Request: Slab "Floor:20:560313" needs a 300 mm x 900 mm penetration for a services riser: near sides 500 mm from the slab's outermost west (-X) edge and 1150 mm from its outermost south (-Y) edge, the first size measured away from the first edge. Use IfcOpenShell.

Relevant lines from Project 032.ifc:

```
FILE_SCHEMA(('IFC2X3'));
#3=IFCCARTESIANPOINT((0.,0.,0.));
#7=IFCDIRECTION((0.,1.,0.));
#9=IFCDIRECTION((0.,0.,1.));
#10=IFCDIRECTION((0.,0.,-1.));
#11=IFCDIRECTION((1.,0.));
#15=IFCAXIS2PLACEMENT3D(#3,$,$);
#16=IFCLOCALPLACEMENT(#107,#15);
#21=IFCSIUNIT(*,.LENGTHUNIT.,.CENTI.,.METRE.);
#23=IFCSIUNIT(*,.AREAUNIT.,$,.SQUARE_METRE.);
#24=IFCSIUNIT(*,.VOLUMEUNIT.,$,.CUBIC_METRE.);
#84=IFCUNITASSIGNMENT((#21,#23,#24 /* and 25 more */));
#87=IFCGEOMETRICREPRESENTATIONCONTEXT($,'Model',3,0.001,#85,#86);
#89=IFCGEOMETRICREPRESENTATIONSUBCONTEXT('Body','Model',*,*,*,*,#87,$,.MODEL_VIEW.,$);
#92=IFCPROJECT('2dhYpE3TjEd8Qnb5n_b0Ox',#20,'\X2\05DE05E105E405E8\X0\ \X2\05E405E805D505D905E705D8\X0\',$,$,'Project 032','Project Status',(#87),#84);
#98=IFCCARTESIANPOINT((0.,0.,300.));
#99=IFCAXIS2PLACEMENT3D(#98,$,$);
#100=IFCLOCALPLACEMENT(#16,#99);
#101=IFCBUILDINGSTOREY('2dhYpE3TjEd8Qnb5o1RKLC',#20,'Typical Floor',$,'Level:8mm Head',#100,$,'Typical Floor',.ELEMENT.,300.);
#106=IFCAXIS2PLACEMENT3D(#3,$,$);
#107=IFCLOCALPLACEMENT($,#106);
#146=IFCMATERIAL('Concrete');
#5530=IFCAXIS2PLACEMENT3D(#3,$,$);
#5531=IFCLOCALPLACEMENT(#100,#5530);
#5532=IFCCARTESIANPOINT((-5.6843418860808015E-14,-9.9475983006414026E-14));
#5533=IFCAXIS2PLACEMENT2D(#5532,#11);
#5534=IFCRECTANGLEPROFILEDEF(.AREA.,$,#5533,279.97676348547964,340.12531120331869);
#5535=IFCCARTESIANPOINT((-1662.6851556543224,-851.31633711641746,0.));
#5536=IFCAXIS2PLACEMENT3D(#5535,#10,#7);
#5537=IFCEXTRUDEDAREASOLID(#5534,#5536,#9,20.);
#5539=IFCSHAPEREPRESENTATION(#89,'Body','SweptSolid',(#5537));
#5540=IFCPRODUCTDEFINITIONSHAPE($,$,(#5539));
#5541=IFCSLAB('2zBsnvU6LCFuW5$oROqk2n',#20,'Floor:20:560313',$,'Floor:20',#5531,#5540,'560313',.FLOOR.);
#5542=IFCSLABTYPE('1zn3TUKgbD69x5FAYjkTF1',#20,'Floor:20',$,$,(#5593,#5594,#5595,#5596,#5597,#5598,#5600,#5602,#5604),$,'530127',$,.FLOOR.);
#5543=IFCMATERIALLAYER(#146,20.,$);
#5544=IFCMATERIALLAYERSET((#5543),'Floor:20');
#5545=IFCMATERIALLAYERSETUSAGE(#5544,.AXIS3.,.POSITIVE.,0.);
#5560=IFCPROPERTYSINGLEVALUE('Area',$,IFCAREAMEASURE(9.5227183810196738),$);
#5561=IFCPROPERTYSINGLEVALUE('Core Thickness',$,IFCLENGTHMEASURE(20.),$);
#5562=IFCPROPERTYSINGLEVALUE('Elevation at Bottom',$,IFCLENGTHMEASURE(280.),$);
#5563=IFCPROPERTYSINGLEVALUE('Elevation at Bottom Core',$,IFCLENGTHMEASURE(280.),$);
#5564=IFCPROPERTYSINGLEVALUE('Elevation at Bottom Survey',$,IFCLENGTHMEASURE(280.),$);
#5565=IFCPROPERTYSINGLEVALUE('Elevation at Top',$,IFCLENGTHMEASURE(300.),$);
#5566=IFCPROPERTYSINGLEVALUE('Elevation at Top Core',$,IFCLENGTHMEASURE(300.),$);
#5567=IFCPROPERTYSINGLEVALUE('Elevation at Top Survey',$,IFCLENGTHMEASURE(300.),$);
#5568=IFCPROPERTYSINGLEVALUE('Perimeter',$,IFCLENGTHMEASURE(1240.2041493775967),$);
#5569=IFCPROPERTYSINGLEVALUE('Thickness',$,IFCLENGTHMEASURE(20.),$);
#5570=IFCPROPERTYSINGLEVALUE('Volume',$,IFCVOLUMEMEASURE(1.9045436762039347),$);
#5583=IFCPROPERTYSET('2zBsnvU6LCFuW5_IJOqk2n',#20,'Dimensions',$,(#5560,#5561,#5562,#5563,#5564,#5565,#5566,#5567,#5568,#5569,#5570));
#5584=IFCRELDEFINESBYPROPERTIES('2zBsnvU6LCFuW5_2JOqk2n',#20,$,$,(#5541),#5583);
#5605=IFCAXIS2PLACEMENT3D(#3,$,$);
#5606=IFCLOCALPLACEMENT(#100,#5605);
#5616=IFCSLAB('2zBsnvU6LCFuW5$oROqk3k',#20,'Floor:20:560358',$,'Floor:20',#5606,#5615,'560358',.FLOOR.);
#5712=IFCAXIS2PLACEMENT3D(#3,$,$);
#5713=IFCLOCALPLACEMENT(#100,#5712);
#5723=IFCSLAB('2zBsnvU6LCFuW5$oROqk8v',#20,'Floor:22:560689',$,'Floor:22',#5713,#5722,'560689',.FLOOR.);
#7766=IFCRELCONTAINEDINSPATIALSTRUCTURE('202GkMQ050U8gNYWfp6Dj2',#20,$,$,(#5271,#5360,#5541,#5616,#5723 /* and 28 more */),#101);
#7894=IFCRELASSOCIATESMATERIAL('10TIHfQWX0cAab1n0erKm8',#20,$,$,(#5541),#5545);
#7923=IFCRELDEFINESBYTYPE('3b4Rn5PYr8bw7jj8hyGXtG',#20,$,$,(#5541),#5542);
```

```python
import numpy as np
import ifcopenshell
import ifcopenshell.api.feature
import ifcopenshell.api.geometry
import ifcopenshell.api.pset
import ifcopenshell.api.root
import ifcopenshell.geom
import ifcopenshell.util.element
import ifcopenshell.util.placement
import ifcopenshell.util.representation
import ifcopenshell.util.shape
import ifcopenshell.util.unit

model = ifcopenshell.open("Project 032.ifc")
unit_scale = ifcopenshell.util.unit.calculate_unit_scale(model)
area_scale = ifcopenshell.util.unit.calculate_unit_scale(model, "AREAUNIT")
volume_scale = ifcopenshell.util.unit.calculate_unit_scale(model, "VOLUMEUNIT")
settings = ifcopenshell.geom.settings()


def volume(element):
    """Net volume in cubic metres, openings subtracted."""
    shape = ifcopenshell.geom.create_shape(settings, element)
    return ifcopenshell.util.shape.get_volume(shape.geometry)


slab = model.by_guid("2zBsnvU6LCFuW5$oROqk2n")
before = volume(slab)

# Extent in the slab's own axes, in metres. The edges named are its -X and -Y sides.
slab_shape = ifcopenshell.geom.create_shape(settings, slab)
vertices = ifcopenshell.util.shape.get_vertices(slab_shape.geometry)
x_min, y_min, bottom = vertices.min(axis=0)
top = vertices[:, 2].max()

opening = ifcopenshell.api.root.create_entity(model, ifc_class="IfcOpeningElement", name="Services riser opening")
context = ifcopenshell.util.representation.get_context(model, "Model", "Body", "MODEL_VIEW")
width, depth = 0.3, 0.9
outline = [(0.0, 0.0), (width, 0.0), (width, depth), (0.0, depth), (0.0, 0.0)]
# Overshoot both faces by 50 mm so the cut is clean.
shape = ifcopenshell.api.geometry.add_slab_representation(
    model, context=context, depth=top - bottom + 0.1, polyline=outline
)
ifcopenshell.api.geometry.assign_representation(model, product=opening, representation=shape)

matrix = ifcopenshell.util.placement.get_local_placement(slab.ObjectPlacement)
matrix[:, 3] = matrix @ np.append(np.array([x_min + 0.5, y_min + 1.15, bottom - 0.05]) / unit_scale, 1.0)
ifcopenshell.api.geometry.edit_object_placement(model, product=opening, matrix=matrix, is_si=False)
ifcopenshell.api.feature.add_feature(model, feature=opening, element=slab)

after = volume(slab)

# Update the slab's stored quantities.
pset = model.by_id(ifcopenshell.util.element.get_pset(slab, "Dimensions", should_inherit=False)["id"])
ifcopenshell.api.pset.edit_pset(model, pset=pset, properties={
    "Area": model.create_entity("IfcAreaMeasure", after / (top - bottom) / area_scale),
    "Volume": model.create_entity("IfcVolumeMeasure", after / volume_scale),
})

print(f"slab volume {before:.3f} -> {after:.3f} m3")

model.write("Project 032_updated.ifc")
```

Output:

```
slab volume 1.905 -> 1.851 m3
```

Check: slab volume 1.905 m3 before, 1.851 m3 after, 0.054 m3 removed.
